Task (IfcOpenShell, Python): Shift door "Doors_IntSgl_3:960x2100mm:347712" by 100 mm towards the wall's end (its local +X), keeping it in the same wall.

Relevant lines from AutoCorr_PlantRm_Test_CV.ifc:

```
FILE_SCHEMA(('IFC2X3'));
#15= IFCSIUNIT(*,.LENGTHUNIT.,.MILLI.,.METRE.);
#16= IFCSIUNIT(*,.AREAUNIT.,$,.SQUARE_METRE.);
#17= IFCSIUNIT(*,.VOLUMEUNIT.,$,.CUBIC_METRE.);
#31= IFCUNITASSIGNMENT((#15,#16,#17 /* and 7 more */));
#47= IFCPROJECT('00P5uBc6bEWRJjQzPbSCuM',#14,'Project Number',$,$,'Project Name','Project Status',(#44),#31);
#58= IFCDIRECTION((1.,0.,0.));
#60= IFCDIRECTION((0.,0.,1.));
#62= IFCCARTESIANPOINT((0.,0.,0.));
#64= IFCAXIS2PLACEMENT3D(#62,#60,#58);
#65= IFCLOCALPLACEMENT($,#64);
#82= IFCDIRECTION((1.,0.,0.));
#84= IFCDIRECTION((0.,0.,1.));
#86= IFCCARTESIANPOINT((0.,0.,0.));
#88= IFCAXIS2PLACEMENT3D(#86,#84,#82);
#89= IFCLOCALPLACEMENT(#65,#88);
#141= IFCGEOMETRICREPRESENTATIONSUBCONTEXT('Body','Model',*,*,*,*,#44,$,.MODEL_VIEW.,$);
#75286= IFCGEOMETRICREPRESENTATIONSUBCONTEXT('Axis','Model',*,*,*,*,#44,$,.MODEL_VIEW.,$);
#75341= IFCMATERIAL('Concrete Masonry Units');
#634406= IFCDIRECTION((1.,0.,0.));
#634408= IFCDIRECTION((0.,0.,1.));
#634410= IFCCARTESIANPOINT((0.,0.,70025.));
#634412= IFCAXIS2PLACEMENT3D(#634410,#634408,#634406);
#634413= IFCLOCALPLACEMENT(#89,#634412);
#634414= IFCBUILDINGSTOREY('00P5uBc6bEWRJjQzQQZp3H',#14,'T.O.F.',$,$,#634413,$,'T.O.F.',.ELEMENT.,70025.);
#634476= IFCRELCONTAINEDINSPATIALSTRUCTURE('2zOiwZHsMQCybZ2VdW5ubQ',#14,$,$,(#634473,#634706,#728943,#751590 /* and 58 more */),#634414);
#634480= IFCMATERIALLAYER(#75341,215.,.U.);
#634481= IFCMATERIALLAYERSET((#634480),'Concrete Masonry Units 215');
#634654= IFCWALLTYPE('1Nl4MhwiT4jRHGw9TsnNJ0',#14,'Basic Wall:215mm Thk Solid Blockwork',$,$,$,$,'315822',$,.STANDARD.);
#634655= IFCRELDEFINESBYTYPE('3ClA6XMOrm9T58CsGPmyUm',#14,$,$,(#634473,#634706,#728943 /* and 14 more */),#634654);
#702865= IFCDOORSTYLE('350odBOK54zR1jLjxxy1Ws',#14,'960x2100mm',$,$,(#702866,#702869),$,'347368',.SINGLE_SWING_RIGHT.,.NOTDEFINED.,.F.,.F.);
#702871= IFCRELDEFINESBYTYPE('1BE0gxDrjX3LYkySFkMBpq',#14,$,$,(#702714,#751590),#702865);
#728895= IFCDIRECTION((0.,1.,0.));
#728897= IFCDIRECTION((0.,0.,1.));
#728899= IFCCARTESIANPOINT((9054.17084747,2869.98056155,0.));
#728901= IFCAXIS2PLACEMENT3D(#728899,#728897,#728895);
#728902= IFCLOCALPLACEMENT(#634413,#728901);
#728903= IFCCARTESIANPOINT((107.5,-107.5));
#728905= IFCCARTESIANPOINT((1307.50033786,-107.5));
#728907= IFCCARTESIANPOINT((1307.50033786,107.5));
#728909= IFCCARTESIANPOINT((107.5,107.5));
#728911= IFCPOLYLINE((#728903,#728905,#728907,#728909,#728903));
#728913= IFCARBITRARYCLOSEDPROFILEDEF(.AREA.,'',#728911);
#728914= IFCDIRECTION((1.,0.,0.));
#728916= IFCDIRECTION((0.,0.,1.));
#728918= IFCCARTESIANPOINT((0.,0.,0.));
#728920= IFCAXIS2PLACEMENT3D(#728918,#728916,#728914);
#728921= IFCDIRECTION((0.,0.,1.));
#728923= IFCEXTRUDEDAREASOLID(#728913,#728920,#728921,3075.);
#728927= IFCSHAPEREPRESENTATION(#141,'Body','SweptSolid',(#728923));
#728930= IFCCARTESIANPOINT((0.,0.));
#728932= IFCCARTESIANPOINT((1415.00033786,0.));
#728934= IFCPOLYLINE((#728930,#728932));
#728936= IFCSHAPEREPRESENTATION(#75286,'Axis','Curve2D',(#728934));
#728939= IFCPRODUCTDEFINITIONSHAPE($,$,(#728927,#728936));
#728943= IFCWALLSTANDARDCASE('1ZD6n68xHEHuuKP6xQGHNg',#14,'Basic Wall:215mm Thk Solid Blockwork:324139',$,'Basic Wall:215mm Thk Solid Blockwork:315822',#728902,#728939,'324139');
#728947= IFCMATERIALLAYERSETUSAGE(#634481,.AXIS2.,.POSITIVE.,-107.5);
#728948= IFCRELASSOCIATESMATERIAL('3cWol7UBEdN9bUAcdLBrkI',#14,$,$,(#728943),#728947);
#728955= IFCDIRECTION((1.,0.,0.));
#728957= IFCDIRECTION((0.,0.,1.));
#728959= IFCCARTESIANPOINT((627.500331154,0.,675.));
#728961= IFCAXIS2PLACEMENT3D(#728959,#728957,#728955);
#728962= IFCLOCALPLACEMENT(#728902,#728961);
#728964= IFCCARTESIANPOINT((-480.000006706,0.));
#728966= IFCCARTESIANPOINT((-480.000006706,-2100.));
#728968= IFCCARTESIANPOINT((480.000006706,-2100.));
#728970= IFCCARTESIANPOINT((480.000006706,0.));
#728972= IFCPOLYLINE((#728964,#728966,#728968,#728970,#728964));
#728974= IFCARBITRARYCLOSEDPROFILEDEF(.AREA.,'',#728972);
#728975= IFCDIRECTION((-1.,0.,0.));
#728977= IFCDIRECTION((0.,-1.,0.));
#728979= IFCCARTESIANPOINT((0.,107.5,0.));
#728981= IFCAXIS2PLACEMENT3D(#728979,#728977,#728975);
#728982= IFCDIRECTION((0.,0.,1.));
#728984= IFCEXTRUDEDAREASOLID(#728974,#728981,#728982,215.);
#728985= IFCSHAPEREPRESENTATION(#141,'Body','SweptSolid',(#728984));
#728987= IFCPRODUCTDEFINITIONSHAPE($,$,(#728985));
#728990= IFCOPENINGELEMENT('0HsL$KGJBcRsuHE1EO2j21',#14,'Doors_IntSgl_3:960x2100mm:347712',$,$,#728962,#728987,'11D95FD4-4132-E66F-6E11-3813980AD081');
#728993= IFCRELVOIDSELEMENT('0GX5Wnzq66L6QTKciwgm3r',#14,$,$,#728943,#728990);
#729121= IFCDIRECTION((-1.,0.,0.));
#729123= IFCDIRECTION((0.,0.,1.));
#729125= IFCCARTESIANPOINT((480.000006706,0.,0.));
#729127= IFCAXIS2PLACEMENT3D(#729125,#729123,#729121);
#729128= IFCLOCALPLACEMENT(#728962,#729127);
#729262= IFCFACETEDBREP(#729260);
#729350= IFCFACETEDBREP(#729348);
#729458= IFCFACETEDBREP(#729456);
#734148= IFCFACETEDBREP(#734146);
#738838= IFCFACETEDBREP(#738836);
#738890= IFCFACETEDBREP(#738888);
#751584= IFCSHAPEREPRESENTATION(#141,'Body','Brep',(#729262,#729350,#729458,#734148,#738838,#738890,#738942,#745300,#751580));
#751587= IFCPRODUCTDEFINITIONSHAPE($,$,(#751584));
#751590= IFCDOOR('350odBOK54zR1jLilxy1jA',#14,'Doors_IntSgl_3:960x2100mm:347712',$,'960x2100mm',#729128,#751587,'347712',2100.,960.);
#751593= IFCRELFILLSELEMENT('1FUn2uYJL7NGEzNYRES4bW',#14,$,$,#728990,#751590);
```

```python
import ifcopenshell
import ifcopenshell.api.geometry
import ifcopenshell.util.placement

model = ifcopenshell.open("AutoCorr_PlantRm_Test_CV.ifc")

door = model.by_guid("350odBOK54zR1jLilxy1jA")
opening = door.FillsVoids[0].RelatingOpeningElement
wall = opening.VoidsElements[0].RelatingBuildingElement

wall_matrix = ifcopenshell.util.placement.get_local_placement(wall.ObjectPlacement)
shift = wall_matrix[:3, 0] * 100.0
before = ifcopenshell.util.placement.get_local_placement(door.ObjectPlacement)[:3, 3].copy()

# The door is placed relative to its opening, so it follows when the opening moves.
matrix = ifcopenshell.util.placement.get_local_placement(opening.ObjectPlacement)
matrix[:3, 3] += shift
ifcopenshell.api.geometry.edit_object_placement(
    model, product=opening, matrix=matrix, is_si=False, should_transform_children=True
)

after = ifcopenshell.util.placement.get_local_placement(door.ObjectPlacement)[:3, 3]
print("door moved by", (after - before).round(3) + 0.0)

model.write("AutoCorr_PlantRm_Test_CV-out.ifc")
```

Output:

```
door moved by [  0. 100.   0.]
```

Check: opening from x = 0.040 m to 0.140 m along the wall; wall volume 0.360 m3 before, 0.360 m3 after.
